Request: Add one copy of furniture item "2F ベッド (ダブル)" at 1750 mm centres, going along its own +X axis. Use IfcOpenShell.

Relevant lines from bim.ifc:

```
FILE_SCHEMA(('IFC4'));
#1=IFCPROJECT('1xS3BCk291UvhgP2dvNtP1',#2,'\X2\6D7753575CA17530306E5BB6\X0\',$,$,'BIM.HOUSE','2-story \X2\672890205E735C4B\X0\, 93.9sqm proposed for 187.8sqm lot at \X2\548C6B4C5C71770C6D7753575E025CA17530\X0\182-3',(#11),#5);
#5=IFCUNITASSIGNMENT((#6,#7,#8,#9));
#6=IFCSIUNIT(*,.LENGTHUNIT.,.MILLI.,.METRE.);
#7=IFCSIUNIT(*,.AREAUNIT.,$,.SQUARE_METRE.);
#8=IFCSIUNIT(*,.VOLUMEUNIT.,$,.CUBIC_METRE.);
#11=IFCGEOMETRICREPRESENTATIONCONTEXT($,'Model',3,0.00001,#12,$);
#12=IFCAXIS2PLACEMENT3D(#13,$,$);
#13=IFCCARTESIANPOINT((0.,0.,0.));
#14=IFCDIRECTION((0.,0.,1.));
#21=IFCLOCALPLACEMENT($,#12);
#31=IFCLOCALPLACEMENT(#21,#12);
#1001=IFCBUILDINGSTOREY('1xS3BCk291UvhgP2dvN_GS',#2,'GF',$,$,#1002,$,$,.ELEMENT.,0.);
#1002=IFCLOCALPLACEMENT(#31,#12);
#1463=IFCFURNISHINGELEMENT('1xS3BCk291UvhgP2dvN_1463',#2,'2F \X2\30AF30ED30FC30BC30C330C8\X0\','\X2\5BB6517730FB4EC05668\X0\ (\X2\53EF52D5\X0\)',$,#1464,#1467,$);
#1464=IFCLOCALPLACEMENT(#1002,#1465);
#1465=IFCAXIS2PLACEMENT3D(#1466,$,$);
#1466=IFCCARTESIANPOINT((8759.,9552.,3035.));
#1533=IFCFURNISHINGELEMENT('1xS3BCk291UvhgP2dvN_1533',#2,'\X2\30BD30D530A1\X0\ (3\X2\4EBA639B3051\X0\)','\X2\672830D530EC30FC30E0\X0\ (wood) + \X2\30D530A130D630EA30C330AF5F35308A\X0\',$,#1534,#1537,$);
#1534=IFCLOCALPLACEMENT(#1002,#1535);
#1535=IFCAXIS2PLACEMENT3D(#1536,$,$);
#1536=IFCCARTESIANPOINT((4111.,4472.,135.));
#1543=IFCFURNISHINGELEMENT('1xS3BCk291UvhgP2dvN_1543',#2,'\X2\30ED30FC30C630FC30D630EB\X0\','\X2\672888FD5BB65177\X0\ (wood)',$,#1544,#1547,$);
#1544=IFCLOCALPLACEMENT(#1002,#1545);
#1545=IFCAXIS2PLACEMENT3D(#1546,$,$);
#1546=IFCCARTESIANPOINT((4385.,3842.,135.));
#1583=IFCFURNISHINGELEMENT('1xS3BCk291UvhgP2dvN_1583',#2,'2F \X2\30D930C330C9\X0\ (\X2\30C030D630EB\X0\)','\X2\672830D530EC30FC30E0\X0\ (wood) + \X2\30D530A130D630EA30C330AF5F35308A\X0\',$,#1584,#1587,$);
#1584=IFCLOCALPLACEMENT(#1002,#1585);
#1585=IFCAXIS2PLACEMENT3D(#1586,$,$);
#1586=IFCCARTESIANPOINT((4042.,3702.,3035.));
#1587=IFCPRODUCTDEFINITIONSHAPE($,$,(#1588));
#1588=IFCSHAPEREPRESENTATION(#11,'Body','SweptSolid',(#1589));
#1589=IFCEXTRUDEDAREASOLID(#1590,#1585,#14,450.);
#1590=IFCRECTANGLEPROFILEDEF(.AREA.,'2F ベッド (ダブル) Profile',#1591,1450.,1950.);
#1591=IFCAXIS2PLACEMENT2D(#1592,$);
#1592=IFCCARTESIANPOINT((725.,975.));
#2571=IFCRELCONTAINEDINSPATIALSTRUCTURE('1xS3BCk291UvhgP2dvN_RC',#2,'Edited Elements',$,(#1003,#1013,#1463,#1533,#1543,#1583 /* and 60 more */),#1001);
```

```python
import ifcopenshell
import ifcopenshell.api.geometry
import ifcopenshell.api.root
import ifcopenshell.util.element
import ifcopenshell.util.placement

model = ifcopenshell.open("bim.ifc")


def reuse_history(source, copy):
    """copy_class also copies each property set's owner history, people and application; keep the originals."""
    for rel in copy.IsDefinedBy:
        if rel.is_a("IfcRelDefinesByProperties") and (history := rel.RelatingPropertyDefinition.OwnerHistory):
            rel.RelatingPropertyDefinition.OwnerHistory = source.OwnerHistory
            ifcopenshell.util.element.remove_deep2(model, history)


source = model.by_guid("1xS3BCk291UvhgP2dvN_1583")
base = ifcopenshell.util.placement.get_local_placement(source.ObjectPlacement)
step = base[:3, 0] * 1750.0

for i in range(1, 2):
    copy = ifcopenshell.api.root.copy_class(model, product=source)
    copy.Representation = ifcopenshell.util.element.copy_deep(
        model, source.Representation, exclude=["IfcGeometricRepresentationContext", "IfcRepresentationMap"]
    )
    reuse_history(source, copy)
    matrix = base.copy()
    matrix[:3, 3] += i * step
    print("added at", matrix[:3, 3].round(3) + 0.0)
    ifcopenshell.api.geometry.edit_object_placement(model, product=copy, matrix=matrix, is_si=False)

model.write("bim_rev.ifc")
```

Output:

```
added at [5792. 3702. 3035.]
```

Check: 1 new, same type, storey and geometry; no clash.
